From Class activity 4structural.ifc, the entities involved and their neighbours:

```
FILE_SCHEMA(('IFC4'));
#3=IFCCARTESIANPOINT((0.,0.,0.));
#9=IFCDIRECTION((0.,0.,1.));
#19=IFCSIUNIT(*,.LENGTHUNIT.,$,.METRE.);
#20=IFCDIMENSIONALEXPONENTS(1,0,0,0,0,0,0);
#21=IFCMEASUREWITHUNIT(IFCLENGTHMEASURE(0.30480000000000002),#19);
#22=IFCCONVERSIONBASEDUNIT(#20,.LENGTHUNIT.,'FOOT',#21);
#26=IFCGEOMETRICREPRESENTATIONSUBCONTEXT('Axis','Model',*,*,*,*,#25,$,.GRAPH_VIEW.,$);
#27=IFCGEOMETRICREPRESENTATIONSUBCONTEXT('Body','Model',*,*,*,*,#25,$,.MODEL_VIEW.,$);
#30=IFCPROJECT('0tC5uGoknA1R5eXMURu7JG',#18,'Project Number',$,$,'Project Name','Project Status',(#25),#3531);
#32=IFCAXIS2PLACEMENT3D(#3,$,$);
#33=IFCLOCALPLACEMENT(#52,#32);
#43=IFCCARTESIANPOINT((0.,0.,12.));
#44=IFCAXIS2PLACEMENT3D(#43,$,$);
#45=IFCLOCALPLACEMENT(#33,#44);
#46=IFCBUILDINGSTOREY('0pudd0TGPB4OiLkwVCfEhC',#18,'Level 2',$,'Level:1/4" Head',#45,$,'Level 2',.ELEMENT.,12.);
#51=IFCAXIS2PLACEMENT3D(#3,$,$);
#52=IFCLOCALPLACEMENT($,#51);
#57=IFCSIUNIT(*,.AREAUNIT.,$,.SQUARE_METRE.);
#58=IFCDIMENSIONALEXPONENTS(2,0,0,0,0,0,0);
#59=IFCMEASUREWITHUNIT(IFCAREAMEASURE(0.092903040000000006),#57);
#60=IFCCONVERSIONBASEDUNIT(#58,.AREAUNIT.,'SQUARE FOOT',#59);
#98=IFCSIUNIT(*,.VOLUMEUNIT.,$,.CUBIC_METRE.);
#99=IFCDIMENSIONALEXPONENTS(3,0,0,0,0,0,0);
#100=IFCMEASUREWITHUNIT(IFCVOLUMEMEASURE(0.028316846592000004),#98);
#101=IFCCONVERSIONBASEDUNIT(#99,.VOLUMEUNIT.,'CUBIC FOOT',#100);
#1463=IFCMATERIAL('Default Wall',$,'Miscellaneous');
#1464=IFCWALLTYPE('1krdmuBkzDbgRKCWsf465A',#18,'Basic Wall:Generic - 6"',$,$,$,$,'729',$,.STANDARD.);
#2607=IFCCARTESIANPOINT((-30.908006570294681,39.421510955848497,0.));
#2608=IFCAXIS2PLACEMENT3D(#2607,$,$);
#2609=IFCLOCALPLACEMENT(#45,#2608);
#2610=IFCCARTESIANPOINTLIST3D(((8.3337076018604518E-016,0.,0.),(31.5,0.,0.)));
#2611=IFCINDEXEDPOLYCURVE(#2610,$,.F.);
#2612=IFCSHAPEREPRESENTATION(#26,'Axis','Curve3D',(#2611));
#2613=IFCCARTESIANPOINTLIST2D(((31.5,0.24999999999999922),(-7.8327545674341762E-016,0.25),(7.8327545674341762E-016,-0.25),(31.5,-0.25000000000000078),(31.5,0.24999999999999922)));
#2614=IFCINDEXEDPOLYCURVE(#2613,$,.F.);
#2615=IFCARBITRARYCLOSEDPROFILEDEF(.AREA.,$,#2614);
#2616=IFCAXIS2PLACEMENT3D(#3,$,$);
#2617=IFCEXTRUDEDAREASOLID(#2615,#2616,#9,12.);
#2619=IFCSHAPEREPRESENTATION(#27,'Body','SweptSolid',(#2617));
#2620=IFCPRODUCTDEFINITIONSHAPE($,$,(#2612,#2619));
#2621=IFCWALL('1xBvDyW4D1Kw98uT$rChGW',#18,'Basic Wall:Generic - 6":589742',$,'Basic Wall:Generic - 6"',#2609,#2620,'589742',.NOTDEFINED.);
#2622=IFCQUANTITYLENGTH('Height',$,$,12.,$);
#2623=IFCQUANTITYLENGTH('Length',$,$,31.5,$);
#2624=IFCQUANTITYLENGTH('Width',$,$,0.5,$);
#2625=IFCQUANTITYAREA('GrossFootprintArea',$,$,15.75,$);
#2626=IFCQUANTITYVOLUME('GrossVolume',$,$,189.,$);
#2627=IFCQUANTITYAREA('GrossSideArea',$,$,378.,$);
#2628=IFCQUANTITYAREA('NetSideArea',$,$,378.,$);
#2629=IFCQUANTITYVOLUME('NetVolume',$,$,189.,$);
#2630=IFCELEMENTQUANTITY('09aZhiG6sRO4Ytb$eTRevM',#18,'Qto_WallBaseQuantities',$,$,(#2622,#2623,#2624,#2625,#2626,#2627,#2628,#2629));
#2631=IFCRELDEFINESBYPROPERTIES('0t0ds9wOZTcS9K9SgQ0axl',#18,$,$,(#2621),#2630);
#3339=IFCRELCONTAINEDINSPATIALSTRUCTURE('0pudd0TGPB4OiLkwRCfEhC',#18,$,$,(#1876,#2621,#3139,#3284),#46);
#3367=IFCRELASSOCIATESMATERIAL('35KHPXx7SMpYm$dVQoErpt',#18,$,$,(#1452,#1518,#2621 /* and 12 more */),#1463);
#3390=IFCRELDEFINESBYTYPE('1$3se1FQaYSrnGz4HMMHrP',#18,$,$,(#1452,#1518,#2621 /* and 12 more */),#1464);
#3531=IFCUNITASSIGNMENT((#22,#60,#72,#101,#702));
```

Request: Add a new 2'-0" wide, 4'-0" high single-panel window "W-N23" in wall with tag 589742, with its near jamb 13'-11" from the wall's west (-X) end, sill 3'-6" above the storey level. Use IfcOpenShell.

```python
import numpy as np
import ifcopenshell
import ifcopenshell.api.feature
import ifcopenshell.api.geometry
import ifcopenshell.api.pset
import ifcopenshell.api.root
import ifcopenshell.api.spatial
import ifcopenshell.geom
import ifcopenshell.util.element
import ifcopenshell.util.placement
import ifcopenshell.util.representation
import ifcopenshell.util.shape
import ifcopenshell.util.unit

model = ifcopenshell.open("Class activity 4structural.ifc")
unit_scale = ifcopenshell.util.unit.calculate_unit_scale(model)
area_scale = ifcopenshell.util.unit.calculate_unit_scale(model, "AREAUNIT")
volume_scale = ifcopenshell.util.unit.calculate_unit_scale(model, "VOLUMEUNIT")
settings = ifcopenshell.geom.settings()


def volume(element):
    """Net volume in cubic metres, openings subtracted."""
    shape = ifcopenshell.geom.create_shape(settings, element)
    return ifcopenshell.util.shape.get_volume(shape.geometry)


wall = model.by_guid("1xBvDyW4D1Kw98uT$rChGW")
storey = ifcopenshell.util.element.get_container(wall, ifc_class="IfcBuildingStorey")
context = ifcopenshell.util.representation.get_context(model, "Model", "Body", "MODEL_VIEW")
before = volume(wall)

width, height, from_end, sill = 0.6096, 1.2192, 4.2418, 1.0668  # metres

# The wall runs along its own X axis, and the end named is its -X end.
wall_shape = ifcopenshell.geom.create_shape(settings, wall)
x, y, z = ifcopenshell.util.shape.get_vertices(wall_shape.geometry).T
start = x.min() + from_end
face, thickness = float(y.min()), float(y.max() - y.min())
wall_matrix = ifcopenshell.util.placement.get_local_placement(wall.ObjectPlacement)
level = ifcopenshell.util.placement.get_local_placement(storey.ObjectPlacement)[2, 3]


def in_wall(x, y):
    """Placement at x, y metres in the wall's axes, at sill height."""
    matrix = wall_matrix.copy()
    matrix[:, 3] = wall_matrix @ np.array([x / unit_scale, y / unit_scale, 0.0, 1.0])
    matrix[2, 3] = level + sill / unit_scale
    return matrix


# Opening: a box that overshoots both wall faces by 50 mm.
opening = ifcopenshell.api.root.create_entity(model, ifc_class="IfcOpeningElement", predefined_type="OPENING")
box = ifcopenshell.api.geometry.add_wall_representation(
    model, context=context, length=width, height=height, thickness=thickness + 0.1
)
ifcopenshell.api.geometry.assign_representation(model, product=opening, representation=box)
ifcopenshell.api.geometry.edit_object_placement(model, product=opening, matrix=in_wall(start, face - 0.05), is_si=False)
ifcopenshell.api.feature.add_feature(model, feature=opening, element=wall)

window = ifcopenshell.api.root.create_entity(model, ifc_class="IfcWindow", name="W-N23", predefined_type="WINDOW")
window.OverallWidth, window.OverallHeight = width / unit_scale, height / unit_scale
window.PartitioningType = "SINGLE_PANEL"
body = ifcopenshell.api.geometry.add_window_representation(
    model,
    context=context,
    overall_width=window.OverallWidth,
    overall_height=window.OverallHeight,
    partition_type="SINGLE_PANEL",
)
ifcopenshell.api.geometry.assign_representation(model, product=window, representation=body)
ifcopenshell.api.spatial.assign_container(model, products=[window], relating_structure=storey)
ifcopenshell.api.feature.add_filling(model, opening=opening, element=window)

# Centre the window in the wall's thickness.
ifcopenshell.api.geometry.edit_object_placement(model, product=window, matrix=in_wall(start, face), is_si=False)
window_shape = ifcopenshell.geom.create_shape(settings, window)
depth = ifcopenshell.util.shape.get_vertices(window_shape.geometry)[:, 1]
offset = face + thickness / 2 - (depth.min() + depth.max()) / 2
ifcopenshell.api.geometry.edit_object_placement(model, product=window, matrix=in_wall(start, offset), is_si=False)

after = volume(wall)

# Update the wall's stored quantities.
qto = model.by_id(ifcopenshell.util.element.get_pset(wall, "Qto_WallBaseQuantities", should_inherit=False)["id"])
ifcopenshell.api.pset.edit_qto(model, qto=qto, properties={
    "NetSideArea": after / thickness / area_scale,
    "NetVolume": after / volume_scale,
})

print(f"wall volume {before:.3f} -> {after:.3f} m3")

model.write("Class activity 4structural_v2.ifc")
```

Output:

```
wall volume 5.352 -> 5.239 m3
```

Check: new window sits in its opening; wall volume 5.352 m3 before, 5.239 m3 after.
